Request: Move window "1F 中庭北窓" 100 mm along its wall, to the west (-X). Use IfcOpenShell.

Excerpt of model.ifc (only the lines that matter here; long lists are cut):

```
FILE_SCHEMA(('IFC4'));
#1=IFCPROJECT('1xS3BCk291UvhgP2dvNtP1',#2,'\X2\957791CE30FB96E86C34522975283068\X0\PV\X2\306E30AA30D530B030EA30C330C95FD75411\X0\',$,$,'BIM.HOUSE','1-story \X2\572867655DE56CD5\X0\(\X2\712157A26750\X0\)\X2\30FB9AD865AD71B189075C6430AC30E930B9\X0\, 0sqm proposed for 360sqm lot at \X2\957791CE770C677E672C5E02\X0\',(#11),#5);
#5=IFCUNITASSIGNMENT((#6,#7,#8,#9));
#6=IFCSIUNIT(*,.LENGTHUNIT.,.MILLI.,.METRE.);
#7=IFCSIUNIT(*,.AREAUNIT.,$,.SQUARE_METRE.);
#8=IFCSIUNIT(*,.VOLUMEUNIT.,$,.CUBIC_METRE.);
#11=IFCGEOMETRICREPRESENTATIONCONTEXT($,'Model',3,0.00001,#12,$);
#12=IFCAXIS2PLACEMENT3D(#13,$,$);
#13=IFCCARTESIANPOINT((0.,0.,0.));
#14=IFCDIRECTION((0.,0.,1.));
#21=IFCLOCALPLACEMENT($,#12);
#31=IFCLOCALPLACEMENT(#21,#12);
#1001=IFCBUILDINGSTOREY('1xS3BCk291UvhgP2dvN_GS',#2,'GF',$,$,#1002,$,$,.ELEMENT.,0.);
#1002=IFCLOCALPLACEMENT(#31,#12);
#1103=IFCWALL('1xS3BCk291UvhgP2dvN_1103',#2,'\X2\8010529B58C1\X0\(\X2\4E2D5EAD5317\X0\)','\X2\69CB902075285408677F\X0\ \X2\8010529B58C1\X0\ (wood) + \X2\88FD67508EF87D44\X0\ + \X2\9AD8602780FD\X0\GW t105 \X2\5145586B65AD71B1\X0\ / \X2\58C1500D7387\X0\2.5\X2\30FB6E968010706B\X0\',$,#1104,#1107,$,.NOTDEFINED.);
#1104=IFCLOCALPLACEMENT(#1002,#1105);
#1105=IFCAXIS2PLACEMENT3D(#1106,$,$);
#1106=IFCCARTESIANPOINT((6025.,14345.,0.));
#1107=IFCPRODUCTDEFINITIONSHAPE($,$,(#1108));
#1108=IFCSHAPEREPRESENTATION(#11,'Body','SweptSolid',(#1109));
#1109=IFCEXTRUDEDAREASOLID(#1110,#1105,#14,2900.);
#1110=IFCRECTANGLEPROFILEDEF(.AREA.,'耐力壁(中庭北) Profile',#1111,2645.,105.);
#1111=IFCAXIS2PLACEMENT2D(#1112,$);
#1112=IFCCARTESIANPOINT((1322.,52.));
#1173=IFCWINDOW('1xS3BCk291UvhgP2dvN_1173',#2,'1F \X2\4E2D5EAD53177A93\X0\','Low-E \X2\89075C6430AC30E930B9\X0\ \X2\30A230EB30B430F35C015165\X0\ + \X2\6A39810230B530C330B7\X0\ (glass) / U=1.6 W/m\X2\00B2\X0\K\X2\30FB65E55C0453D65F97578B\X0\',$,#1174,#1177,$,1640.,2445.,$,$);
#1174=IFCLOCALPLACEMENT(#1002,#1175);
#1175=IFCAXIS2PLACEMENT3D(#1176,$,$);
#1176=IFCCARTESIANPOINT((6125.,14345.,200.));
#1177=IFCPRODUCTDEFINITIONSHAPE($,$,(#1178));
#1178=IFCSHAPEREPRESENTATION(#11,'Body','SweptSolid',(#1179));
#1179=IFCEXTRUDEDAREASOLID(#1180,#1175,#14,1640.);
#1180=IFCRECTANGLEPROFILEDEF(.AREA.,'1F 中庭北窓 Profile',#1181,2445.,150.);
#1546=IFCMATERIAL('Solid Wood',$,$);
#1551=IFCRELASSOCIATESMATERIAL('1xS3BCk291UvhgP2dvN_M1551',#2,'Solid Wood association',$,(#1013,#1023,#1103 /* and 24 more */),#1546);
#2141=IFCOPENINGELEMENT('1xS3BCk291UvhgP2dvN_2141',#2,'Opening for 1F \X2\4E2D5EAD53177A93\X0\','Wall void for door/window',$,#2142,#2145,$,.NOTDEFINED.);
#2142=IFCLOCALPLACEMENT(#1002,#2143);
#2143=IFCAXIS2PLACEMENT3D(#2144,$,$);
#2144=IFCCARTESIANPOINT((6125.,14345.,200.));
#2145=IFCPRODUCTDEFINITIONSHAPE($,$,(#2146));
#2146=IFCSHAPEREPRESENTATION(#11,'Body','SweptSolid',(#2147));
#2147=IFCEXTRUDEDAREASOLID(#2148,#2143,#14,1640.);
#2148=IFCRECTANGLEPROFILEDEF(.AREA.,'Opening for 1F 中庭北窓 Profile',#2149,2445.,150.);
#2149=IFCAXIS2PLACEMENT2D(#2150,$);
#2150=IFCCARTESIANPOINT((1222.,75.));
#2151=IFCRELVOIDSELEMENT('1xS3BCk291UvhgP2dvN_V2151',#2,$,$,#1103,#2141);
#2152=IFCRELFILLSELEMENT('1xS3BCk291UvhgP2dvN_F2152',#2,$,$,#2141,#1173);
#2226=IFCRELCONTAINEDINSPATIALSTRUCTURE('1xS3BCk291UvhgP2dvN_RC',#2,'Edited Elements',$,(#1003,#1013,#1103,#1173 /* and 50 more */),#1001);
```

```python
import ifcopenshell
import ifcopenshell.api.geometry
import ifcopenshell.util.placement
import ifcopenshell.util.unit

model = ifcopenshell.open("model.ifc")
unit_scale = ifcopenshell.util.unit.calculate_unit_scale(model)

window = model.by_guid("1xS3BCk291UvhgP2dvN_1173")
opening = window.FillsVoids[0].RelatingOpeningElement
wall = opening.VoidsElements[0].RelatingBuildingElement

wall_matrix = ifcopenshell.util.placement.get_local_placement(wall.ObjectPlacement)
shift = wall_matrix[:3, 0] * -0.1 / unit_scale
before = ifcopenshell.util.placement.get_local_placement(window.ObjectPlacement)[:3, 3].copy()

# The window is not placed relative to its opening, so move both.
for product in (opening, window):
    matrix = ifcopenshell.util.placement.get_local_placement(product.ObjectPlacement)
    matrix[:3, 3] += shift
    ifcopenshell.api.geometry.edit_object_placement(model, product=product, matrix=matrix, is_si=False)

after = ifcopenshell.util.placement.get_local_placement(window.ObjectPlacement)[:3, 3]
print("window moved by", (after - before).round(3) + 0.0)

model.write("model_updated.ifc")
```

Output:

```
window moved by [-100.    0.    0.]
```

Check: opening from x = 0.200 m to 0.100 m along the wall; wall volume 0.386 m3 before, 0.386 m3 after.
